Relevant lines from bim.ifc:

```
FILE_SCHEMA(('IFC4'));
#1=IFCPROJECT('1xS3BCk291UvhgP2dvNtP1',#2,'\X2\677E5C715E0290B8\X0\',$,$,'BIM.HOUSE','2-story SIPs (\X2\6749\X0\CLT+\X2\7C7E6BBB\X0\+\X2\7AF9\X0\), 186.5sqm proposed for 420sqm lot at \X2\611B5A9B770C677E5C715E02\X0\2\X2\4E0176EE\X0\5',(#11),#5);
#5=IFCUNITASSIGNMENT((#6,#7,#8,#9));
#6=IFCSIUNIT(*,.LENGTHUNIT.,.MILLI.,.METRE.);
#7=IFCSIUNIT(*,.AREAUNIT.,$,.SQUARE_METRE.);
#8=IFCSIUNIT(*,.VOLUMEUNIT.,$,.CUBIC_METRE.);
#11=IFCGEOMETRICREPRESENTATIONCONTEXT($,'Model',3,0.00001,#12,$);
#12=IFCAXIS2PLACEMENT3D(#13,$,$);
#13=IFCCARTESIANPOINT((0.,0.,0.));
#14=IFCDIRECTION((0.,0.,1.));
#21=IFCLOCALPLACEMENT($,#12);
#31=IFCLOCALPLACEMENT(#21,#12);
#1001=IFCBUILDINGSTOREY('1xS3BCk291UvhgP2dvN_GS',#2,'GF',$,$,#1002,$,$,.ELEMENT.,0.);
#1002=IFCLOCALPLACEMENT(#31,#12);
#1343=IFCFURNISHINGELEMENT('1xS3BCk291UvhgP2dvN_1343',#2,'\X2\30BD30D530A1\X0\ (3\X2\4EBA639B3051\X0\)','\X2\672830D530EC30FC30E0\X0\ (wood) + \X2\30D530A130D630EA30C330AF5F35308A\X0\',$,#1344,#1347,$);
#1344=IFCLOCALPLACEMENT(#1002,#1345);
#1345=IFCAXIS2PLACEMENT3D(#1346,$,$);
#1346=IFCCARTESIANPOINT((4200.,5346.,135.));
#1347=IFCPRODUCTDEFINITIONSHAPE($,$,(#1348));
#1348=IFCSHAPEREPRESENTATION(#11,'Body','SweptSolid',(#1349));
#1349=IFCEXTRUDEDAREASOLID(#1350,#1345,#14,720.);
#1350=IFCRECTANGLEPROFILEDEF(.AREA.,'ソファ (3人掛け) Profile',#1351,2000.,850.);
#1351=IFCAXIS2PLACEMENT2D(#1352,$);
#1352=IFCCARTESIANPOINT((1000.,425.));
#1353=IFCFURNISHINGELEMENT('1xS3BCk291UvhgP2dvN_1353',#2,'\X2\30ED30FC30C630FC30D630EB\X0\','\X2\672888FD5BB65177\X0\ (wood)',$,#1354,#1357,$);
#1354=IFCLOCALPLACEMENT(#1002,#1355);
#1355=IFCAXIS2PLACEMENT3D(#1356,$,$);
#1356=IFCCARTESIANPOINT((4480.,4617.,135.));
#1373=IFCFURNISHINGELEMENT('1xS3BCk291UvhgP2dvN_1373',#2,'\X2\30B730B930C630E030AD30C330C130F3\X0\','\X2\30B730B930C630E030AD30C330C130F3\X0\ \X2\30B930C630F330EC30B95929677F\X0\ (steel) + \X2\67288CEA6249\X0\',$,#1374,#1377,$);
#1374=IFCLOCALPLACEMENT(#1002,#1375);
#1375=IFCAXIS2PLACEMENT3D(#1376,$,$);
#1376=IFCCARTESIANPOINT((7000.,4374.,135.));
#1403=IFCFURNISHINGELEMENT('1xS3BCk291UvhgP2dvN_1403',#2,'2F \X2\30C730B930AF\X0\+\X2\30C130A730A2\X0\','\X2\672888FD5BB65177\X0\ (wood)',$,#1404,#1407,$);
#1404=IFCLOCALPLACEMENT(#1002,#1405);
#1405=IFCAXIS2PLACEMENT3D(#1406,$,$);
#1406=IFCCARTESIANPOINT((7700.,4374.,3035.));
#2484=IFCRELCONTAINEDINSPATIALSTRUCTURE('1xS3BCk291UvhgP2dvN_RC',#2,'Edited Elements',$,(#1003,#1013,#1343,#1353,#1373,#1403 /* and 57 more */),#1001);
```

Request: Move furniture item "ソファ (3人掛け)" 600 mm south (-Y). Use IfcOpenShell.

```python
import ifcopenshell
import ifcopenshell.api.geometry
import ifcopenshell.util.placement

model = ifcopenshell.open("bim.ifc")

item = model.by_id(1343)
matrix = ifcopenshell.util.placement.get_local_placement(item.ObjectPlacement)
matrix[1, 3] -= 600.0
ifcopenshell.api.geometry.edit_object_placement(model, product=item, matrix=matrix, is_si=False)

print(ifcopenshell.util.placement.get_local_placement(item.ObjectPlacement).round(3) + 0.0)

model.write("bim_edited.ifc")
```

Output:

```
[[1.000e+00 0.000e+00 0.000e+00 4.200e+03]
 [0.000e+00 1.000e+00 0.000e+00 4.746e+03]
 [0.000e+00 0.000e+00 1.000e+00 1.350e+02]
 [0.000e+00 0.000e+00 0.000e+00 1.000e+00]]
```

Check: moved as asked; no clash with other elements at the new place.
